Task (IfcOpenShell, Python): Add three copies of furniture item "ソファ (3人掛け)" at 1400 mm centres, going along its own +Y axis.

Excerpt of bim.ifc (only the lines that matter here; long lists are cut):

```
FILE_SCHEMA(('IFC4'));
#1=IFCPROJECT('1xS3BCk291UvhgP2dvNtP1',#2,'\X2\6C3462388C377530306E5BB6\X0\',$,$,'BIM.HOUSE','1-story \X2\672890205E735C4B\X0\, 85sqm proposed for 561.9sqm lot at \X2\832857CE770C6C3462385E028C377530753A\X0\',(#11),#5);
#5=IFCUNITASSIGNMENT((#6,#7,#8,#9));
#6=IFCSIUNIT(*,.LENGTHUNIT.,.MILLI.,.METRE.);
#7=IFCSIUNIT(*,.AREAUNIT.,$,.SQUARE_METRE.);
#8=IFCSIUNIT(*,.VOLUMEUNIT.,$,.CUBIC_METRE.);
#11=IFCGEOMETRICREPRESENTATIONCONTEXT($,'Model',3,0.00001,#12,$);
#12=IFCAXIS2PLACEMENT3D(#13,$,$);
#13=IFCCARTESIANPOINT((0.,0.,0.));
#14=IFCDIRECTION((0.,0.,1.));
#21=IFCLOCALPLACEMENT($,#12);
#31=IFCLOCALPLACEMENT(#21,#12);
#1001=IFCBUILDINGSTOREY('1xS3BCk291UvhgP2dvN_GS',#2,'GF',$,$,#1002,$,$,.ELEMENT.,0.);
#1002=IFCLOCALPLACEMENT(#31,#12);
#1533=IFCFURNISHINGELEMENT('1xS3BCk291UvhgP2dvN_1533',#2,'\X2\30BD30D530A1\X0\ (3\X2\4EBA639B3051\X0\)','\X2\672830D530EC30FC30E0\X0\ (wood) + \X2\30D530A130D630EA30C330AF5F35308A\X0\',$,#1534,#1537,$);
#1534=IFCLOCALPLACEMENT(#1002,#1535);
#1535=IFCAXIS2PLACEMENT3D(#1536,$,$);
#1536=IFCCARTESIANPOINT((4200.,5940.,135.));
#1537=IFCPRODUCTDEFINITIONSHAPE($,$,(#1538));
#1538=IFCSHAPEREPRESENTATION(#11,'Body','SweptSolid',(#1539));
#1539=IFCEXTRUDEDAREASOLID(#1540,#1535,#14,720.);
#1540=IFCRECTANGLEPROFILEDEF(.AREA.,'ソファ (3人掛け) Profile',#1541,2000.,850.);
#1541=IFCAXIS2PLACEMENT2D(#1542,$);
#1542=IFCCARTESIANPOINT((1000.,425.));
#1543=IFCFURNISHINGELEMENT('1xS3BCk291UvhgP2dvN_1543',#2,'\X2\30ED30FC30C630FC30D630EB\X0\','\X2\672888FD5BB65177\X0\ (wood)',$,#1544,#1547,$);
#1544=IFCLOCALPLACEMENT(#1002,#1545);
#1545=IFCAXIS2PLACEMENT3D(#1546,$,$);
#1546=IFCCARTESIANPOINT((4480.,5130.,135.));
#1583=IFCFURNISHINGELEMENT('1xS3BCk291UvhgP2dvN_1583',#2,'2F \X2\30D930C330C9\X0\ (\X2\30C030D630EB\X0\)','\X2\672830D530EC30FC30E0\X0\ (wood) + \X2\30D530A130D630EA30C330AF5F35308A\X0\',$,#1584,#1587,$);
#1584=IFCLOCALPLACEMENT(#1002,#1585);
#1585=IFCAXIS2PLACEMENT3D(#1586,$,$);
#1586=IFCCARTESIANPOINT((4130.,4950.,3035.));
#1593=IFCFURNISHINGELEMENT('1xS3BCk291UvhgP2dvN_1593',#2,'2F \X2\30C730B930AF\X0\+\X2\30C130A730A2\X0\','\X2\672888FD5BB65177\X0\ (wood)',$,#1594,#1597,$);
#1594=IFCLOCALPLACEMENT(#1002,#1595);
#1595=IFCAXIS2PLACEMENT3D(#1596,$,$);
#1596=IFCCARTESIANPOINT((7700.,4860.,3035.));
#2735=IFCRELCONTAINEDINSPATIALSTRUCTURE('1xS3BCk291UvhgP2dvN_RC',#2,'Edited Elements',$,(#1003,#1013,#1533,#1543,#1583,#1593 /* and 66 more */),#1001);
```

```python
import ifcopenshell
import ifcopenshell.api.geometry
import ifcopenshell.api.root
import ifcopenshell.util.element
import ifcopenshell.util.placement
import ifcopenshell.util.unit

model = ifcopenshell.open("bim.ifc")
unit_scale = ifcopenshell.util.unit.calculate_unit_scale(model)


def reuse_history(source, copy):
    """copy_class also copies each property set's owner history, people and application; keep the originals."""
    for rel in copy.IsDefinedBy:
        if rel.is_a("IfcRelDefinesByProperties") and (history := rel.RelatingPropertyDefinition.OwnerHistory):
            rel.RelatingPropertyDefinition.OwnerHistory = source.OwnerHistory
            ifcopenshell.util.element.remove_deep2(model, history)


source = model.by_guid("1xS3BCk291UvhgP2dvN_1533")
base = ifcopenshell.util.placement.get_local_placement(source.ObjectPlacement)
step = base[:3, 1] * 1.4 / unit_scale

for i in range(1, 4):
    copy = ifcopenshell.api.root.copy_class(model, product=source)
    copy.Representation = ifcopenshell.util.element.copy_deep(
        model, source.Representation, exclude=["IfcGeometricRepresentationContext", "IfcRepresentationMap"]
    )
    reuse_history(source, copy)
    matrix = base.copy()
    matrix[:3, 3] += i * step
    print("added at", matrix[:3, 3].round(3) + 0.0)
    ifcopenshell.api.geometry.edit_object_placement(model, product=copy, matrix=matrix, is_si=False)

model.write("bim_updated.ifc")
```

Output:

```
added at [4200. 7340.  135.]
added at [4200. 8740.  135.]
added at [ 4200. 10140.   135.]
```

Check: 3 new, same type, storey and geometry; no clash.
